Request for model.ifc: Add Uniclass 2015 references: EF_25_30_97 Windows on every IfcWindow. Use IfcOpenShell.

First a look at what the model holds.

```python
import ifcopenshell

model = ifcopenshell.open("model.ifc")
print(model.schema)
print("classifications:", [c.Name for c in model.by_type("IfcClassification")])
for ifc_class in ("IfcDoor", "IfcRoof", "IfcStair", "IfcWall", "IfcWindow"):
    print(ifc_class, len(model.by_type(ifc_class)))
```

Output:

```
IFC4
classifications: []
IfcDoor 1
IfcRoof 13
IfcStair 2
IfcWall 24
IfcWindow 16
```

```python
import ifcopenshell
import ifcopenshell.api.classification

model = ifcopenshell.open("model.ifc")

system = ifcopenshell.api.classification.add_classification(model, classification="Uniclass 2015")

codes = {
    "IfcWindow": ("EF_25_30_97", "Windows"),
}
for ifc_class, (code, name) in codes.items():
    products = model.by_type(ifc_class)
    ifcopenshell.api.classification.add_reference(
        model, products=products, classification=system, identification=code, name=name
    )
    print(code, len(products))

model.write("model_v2.ifc")
```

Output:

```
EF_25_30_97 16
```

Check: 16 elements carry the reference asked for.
